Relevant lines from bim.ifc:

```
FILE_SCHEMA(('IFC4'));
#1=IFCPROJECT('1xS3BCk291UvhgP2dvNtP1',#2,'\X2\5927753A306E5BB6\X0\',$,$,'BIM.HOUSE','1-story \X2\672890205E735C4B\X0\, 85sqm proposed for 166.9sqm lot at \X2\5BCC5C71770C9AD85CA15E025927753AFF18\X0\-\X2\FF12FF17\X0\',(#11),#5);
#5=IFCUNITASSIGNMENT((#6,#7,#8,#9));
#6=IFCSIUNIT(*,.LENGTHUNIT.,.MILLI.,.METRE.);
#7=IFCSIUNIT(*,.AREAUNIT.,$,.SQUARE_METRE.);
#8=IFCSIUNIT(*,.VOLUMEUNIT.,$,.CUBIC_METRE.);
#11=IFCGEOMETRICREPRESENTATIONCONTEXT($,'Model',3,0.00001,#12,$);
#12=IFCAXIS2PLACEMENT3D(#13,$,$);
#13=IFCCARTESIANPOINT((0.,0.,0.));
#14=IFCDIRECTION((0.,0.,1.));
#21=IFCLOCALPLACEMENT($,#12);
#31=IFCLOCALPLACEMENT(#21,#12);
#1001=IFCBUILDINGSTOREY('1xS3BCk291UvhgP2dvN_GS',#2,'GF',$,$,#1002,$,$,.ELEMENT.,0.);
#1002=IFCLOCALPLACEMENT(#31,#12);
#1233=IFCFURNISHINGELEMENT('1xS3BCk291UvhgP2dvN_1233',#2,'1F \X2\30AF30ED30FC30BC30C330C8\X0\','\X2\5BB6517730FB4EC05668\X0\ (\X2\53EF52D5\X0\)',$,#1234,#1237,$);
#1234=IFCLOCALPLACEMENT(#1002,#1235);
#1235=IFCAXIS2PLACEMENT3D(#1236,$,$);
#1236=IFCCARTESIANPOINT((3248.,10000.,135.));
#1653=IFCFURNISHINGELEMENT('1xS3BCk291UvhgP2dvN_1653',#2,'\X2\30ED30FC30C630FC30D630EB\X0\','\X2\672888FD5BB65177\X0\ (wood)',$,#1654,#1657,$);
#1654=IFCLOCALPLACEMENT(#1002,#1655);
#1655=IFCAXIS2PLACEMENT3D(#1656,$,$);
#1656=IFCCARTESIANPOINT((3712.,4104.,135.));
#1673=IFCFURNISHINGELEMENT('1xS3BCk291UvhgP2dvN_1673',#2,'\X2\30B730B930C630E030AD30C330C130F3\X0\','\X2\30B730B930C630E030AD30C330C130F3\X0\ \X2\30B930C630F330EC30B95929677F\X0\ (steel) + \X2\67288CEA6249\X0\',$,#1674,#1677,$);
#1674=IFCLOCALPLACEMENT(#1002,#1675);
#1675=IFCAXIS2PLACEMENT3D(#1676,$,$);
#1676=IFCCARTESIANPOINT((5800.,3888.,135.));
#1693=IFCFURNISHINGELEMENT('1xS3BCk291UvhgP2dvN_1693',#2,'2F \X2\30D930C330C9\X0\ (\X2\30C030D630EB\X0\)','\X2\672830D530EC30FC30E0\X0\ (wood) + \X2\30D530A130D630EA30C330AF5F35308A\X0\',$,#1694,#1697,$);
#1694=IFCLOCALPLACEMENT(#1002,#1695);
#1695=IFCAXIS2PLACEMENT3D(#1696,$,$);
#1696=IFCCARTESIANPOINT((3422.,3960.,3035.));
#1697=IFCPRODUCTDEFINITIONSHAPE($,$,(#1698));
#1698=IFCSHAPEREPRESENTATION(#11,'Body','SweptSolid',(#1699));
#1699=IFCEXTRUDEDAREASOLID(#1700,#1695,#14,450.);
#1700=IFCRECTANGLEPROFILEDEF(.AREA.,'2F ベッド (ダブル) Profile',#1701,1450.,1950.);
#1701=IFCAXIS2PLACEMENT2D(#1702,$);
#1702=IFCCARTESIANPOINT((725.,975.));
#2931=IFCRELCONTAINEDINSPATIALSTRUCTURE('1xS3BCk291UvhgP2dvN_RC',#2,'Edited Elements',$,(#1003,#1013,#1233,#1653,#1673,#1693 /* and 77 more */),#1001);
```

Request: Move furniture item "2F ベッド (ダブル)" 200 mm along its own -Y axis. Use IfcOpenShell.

```python
import ifcopenshell
import ifcopenshell.api.geometry
import ifcopenshell.util.placement
import ifcopenshell.util.unit

model = ifcopenshell.open("bim.ifc")
unit_scale = ifcopenshell.util.unit.calculate_unit_scale(model)

item = model.by_id(1693)
matrix = ifcopenshell.util.placement.get_local_placement(item.ObjectPlacement)
matrix[:3, 3] -= matrix[:3, 1] * 0.2 / unit_scale
ifcopenshell.api.geometry.edit_object_placement(model, product=item, matrix=matrix, is_si=False)

print(ifcopenshell.util.placement.get_local_placement(item.ObjectPlacement).round(3) + 0.0)

model.write("bim_v2.ifc")
```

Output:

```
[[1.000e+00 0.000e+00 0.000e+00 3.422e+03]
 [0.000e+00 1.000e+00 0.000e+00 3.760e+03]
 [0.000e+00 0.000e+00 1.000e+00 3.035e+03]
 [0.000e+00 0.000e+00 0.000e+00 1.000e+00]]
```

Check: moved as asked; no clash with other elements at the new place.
